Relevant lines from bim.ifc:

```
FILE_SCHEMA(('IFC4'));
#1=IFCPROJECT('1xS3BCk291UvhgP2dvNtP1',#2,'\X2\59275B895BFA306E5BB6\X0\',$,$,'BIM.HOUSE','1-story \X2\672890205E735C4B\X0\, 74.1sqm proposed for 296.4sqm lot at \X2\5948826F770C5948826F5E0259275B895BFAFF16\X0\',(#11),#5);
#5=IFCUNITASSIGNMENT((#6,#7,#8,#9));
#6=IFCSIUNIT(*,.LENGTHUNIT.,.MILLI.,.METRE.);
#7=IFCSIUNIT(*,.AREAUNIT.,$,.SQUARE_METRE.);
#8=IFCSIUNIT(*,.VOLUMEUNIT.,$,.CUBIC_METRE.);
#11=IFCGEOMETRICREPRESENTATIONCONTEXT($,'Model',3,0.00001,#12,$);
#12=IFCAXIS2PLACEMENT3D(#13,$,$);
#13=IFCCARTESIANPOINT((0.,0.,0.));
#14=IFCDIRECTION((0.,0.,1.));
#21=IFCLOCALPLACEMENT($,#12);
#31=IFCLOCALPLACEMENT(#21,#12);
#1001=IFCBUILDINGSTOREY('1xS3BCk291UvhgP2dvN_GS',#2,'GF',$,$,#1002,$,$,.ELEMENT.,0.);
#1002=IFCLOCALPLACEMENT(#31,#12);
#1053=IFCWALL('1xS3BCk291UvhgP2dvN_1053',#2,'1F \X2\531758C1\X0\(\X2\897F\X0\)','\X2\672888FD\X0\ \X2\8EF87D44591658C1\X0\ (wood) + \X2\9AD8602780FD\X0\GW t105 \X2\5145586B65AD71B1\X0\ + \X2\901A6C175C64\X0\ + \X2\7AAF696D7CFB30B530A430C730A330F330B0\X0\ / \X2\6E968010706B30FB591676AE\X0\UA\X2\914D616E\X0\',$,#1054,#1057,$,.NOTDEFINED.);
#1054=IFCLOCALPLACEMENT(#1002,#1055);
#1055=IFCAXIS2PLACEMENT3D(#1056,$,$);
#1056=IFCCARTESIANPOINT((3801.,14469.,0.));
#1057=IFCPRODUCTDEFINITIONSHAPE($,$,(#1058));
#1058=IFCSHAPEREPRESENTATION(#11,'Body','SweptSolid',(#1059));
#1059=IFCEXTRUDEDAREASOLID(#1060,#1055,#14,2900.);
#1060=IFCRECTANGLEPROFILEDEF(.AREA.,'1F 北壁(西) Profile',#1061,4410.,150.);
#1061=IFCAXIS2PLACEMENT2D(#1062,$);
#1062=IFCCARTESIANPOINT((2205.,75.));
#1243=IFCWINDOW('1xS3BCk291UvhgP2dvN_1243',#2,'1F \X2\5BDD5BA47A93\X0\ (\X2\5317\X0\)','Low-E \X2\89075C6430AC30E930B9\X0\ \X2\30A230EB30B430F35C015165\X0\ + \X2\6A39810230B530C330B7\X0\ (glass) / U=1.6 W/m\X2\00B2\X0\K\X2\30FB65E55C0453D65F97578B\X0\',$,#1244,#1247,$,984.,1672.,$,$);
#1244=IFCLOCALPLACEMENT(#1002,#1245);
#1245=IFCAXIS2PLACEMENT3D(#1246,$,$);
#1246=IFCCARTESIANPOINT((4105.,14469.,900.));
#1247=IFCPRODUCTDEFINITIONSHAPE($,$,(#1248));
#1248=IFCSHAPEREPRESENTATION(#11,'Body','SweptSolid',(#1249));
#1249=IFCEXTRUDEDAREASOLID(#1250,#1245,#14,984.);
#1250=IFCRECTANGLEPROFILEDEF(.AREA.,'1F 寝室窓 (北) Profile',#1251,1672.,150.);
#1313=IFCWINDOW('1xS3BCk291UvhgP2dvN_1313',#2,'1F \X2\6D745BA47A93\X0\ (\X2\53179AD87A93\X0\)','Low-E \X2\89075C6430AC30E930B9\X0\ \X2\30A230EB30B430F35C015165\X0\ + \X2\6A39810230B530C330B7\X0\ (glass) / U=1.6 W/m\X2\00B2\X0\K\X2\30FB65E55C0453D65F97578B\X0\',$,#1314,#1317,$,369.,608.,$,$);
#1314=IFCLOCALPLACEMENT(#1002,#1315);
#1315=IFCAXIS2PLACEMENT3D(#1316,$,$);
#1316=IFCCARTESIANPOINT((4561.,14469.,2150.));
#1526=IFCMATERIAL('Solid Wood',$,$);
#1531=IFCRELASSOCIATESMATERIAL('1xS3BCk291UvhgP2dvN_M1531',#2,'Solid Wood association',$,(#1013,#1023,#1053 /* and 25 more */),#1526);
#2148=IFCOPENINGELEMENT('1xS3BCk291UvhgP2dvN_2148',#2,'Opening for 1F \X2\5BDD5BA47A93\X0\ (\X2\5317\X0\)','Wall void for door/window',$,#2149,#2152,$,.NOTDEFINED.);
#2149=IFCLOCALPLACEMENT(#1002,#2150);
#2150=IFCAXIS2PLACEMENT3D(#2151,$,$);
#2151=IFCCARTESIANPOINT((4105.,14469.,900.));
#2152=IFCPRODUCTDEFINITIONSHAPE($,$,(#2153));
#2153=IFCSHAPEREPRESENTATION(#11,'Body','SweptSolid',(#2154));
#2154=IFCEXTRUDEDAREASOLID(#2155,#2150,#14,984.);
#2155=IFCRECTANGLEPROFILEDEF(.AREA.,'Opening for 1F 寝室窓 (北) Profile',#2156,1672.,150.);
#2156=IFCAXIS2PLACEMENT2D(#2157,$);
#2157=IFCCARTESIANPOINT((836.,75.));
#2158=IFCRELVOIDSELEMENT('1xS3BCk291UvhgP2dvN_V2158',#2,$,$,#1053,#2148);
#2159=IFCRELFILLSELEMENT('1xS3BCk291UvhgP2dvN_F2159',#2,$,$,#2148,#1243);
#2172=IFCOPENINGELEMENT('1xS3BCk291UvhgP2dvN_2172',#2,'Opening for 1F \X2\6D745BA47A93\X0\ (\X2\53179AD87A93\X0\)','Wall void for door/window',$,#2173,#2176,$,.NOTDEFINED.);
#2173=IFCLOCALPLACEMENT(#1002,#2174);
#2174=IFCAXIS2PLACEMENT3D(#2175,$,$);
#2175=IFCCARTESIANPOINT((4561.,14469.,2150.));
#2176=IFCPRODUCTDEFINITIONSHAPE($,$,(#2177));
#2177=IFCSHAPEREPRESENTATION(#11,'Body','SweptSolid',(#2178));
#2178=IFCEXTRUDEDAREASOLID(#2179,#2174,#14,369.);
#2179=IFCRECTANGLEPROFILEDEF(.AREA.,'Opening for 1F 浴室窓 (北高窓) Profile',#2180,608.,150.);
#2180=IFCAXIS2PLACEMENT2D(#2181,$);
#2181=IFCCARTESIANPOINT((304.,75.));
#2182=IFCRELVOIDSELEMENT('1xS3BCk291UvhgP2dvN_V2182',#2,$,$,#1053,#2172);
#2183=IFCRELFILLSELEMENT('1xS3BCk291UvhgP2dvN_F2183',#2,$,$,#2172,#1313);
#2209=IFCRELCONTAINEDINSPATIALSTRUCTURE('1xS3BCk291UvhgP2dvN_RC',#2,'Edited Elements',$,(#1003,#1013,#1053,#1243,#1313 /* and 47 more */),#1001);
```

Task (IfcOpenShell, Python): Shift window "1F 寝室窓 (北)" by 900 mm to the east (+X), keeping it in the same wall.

```python
import ifcopenshell
import ifcopenshell.api.geometry
import ifcopenshell.util.placement
import ifcopenshell.util.unit

model = ifcopenshell.open("bim.ifc")
unit_scale = ifcopenshell.util.unit.calculate_unit_scale(model)

window = model.by_guid("1xS3BCk291UvhgP2dvN_1243")
opening = window.FillsVoids[0].RelatingOpeningElement
wall = opening.VoidsElements[0].RelatingBuildingElement

wall_matrix = ifcopenshell.util.placement.get_local_placement(wall.ObjectPlacement)
shift = wall_matrix[:3, 0] * 0.9 / unit_scale
before = ifcopenshell.util.placement.get_local_placement(window.ObjectPlacement)[:3, 3].copy()

# The window is not placed relative to its opening, so move both.
for product in (opening, window):
    matrix = ifcopenshell.util.placement.get_local_placement(product.ObjectPlacement)
    matrix[:3, 3] += shift
    ifcopenshell.api.geometry.edit_object_placement(model, product=product, matrix=matrix, is_si=False)

after = ifcopenshell.util.placement.get_local_placement(window.ObjectPlacement)[:3, 3]
print("window moved by", (after - before).round(3) + 0.0)

model.write("bim_rev.ifc")
```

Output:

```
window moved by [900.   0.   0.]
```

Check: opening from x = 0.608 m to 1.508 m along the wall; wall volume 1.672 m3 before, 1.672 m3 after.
